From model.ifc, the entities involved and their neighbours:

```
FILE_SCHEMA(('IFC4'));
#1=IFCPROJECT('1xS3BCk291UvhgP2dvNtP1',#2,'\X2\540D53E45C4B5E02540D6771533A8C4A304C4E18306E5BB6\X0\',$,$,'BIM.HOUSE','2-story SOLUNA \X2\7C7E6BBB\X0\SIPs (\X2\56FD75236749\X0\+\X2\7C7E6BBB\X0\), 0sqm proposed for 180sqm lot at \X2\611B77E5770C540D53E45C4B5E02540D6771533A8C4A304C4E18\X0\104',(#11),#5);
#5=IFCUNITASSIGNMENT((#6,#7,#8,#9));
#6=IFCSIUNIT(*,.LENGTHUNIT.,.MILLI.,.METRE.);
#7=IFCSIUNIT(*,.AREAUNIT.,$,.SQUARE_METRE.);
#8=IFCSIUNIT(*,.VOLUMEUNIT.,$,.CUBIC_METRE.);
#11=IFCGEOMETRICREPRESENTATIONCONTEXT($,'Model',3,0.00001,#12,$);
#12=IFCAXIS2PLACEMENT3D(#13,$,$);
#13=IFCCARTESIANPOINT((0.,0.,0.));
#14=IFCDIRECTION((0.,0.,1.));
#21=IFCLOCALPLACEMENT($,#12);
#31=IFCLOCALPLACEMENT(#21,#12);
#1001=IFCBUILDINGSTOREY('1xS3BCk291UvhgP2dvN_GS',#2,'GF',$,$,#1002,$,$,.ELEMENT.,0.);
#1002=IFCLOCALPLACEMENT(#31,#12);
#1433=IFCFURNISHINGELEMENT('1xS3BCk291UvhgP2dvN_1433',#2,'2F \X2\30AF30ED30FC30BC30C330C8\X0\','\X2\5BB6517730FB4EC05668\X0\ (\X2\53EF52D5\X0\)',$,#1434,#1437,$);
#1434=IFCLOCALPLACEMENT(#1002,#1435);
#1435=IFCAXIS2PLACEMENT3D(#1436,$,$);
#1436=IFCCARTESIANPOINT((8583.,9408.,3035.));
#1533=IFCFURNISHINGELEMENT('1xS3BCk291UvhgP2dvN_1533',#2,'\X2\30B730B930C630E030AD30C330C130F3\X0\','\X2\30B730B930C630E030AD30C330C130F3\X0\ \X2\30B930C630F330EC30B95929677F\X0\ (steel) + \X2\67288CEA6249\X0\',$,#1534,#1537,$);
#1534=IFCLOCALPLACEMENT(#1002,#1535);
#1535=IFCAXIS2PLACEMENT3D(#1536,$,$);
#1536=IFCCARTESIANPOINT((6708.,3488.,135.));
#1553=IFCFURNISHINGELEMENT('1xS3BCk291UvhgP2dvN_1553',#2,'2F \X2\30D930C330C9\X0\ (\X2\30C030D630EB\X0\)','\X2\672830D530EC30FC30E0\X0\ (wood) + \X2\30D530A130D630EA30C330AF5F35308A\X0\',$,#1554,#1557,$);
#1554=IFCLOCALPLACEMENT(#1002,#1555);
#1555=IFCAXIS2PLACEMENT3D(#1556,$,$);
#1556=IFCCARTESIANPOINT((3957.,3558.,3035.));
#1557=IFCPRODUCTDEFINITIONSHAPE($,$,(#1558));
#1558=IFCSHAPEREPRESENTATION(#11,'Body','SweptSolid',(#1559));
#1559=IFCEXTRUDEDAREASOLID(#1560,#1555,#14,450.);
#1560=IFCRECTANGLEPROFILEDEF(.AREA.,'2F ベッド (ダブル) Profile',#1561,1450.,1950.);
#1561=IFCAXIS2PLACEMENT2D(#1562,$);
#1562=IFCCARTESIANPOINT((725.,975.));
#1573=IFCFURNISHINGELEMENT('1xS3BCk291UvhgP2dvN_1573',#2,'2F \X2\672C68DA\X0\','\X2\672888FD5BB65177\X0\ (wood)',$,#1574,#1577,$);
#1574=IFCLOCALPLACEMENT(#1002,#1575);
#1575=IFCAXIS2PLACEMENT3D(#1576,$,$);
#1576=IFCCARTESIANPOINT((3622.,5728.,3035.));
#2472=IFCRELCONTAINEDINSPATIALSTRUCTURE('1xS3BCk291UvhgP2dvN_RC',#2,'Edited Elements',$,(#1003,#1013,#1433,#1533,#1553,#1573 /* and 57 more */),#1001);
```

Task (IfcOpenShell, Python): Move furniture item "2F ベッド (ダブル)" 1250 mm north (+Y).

```python
import ifcopenshell
import ifcopenshell.api.geometry
import ifcopenshell.util.placement

model = ifcopenshell.open("model.ifc")

item = model.by_guid("1xS3BCk291UvhgP2dvN_1553")
matrix = ifcopenshell.util.placement.get_local_placement(item.ObjectPlacement)
matrix[1, 3] += 1250.0
ifcopenshell.api.geometry.edit_object_placement(model, product=item, matrix=matrix, is_si=False)

print(ifcopenshell.util.placement.get_local_placement(item.ObjectPlacement).round(3) + 0.0)

model.write("model_v2.ifc")
```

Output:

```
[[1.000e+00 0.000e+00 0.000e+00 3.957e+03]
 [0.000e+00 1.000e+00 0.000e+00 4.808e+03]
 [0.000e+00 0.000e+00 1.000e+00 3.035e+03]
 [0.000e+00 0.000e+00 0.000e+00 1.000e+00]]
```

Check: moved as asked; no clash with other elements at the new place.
